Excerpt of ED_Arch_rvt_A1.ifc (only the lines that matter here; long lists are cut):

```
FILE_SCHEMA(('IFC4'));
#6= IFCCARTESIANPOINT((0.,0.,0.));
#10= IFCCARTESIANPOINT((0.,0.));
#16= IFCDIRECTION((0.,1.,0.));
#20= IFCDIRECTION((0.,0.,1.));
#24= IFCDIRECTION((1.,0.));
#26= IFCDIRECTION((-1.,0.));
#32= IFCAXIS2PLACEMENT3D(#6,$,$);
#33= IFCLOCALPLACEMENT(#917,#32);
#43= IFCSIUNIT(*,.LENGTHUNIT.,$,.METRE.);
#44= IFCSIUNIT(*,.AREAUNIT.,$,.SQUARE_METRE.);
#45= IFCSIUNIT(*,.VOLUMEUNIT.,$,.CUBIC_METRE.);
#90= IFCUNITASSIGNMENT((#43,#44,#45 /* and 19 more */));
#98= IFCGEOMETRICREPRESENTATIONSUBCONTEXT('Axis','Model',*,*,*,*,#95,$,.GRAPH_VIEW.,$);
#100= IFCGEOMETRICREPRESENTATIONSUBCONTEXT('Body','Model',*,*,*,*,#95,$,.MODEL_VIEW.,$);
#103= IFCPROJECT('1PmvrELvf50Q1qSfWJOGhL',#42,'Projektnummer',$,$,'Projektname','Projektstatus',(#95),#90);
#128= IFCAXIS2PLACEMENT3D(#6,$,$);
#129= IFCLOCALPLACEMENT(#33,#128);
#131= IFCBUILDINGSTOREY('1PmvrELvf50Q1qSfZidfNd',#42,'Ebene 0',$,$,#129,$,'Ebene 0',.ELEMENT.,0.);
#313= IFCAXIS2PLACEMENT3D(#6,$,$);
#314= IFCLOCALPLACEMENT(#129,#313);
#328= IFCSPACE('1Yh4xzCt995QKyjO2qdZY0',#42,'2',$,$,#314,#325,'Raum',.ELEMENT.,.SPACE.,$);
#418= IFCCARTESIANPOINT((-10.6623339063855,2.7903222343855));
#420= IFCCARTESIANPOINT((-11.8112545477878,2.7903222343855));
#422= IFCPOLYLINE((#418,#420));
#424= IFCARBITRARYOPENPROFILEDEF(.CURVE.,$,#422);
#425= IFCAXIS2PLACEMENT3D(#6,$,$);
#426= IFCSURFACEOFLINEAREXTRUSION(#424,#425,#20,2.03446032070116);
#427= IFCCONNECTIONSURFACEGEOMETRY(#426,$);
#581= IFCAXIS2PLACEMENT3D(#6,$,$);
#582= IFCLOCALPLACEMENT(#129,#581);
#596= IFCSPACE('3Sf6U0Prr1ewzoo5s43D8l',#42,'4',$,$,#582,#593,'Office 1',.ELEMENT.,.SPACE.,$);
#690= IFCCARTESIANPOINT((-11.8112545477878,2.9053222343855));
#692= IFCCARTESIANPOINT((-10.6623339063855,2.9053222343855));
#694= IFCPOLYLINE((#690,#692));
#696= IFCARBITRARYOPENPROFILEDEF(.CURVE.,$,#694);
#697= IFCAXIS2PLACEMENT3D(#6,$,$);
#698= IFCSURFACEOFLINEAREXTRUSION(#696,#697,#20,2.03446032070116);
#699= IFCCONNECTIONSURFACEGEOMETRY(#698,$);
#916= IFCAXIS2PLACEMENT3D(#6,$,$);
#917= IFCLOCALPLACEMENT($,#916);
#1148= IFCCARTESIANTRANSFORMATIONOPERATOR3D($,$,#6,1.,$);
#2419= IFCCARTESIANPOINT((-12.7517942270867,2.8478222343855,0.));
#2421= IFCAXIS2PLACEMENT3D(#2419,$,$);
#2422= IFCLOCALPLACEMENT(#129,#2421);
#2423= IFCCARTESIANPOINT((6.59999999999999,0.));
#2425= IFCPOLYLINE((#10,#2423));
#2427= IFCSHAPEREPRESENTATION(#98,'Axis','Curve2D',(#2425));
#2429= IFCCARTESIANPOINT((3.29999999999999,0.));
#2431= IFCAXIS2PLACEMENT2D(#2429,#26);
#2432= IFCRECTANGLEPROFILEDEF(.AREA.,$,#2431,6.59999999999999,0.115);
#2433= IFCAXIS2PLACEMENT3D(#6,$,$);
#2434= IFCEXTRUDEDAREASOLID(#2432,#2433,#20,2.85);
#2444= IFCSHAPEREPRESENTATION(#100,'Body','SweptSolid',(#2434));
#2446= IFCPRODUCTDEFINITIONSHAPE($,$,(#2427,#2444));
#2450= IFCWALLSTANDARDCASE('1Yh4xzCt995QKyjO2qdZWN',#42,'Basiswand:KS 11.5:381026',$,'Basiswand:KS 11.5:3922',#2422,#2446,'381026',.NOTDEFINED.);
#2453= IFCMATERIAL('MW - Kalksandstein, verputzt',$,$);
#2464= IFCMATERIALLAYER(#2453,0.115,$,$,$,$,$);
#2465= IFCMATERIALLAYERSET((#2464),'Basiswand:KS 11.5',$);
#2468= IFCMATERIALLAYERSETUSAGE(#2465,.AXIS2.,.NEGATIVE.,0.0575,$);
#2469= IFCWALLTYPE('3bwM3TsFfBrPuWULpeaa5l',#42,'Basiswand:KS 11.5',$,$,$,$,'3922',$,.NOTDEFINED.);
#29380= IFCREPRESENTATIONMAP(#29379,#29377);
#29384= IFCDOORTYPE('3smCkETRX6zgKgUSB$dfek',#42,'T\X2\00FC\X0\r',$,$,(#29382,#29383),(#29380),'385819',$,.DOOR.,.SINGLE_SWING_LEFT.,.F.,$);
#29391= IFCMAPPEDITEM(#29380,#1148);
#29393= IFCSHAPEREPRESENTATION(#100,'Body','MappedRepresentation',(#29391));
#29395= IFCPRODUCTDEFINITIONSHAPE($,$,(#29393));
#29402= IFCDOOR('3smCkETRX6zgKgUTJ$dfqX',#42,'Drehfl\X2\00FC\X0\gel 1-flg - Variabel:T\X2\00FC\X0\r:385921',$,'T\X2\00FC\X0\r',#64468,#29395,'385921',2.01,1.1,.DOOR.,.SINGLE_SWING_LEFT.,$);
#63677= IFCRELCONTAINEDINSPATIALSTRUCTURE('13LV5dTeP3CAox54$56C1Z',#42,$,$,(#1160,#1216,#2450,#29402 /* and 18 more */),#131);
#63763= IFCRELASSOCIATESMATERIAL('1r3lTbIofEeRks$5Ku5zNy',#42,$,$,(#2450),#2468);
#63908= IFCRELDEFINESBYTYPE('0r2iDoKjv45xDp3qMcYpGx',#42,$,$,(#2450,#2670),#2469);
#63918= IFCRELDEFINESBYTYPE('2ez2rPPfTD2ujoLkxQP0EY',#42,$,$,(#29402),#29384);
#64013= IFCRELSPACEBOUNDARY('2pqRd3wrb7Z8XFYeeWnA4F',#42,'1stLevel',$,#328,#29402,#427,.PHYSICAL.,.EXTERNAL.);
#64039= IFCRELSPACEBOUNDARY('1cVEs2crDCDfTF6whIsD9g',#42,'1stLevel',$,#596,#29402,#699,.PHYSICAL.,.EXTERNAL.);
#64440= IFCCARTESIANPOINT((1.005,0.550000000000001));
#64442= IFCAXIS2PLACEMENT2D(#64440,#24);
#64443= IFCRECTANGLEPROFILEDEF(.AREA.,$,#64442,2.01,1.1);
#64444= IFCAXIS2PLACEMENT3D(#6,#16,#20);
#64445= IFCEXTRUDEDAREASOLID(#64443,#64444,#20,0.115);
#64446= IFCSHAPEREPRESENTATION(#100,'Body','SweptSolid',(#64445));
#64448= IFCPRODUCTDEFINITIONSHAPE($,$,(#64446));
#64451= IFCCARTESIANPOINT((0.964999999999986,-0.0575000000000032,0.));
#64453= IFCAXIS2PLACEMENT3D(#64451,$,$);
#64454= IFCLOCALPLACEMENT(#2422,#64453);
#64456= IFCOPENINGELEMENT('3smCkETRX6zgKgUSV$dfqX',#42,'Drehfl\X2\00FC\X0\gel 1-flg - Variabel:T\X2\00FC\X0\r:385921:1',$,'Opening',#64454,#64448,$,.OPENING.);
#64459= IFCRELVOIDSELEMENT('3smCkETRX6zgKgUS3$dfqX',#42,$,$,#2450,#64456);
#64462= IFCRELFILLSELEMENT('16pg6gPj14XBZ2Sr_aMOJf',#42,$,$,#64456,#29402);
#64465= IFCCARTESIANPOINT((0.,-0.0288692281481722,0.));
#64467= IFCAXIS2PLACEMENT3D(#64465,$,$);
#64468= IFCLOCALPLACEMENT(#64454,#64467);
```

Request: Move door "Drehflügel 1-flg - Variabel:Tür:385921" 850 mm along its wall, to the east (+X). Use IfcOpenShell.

```python
import numpy as np
import ifcopenshell
import ifcopenshell.api.geometry
import ifcopenshell.util.placement

model = ifcopenshell.open("ED_Arch_rvt_A1.ifc")

door = model.by_id(29402)
opening = door.FillsVoids[0].RelatingOpeningElement
wall = opening.VoidsElements[0].RelatingBuildingElement

wall_matrix = ifcopenshell.util.placement.get_local_placement(wall.ObjectPlacement)
shift = wall_matrix[:3, 0] * 0.85
before = ifcopenshell.util.placement.get_local_placement(door.ObjectPlacement)[:3, 3].copy()

# The door is placed relative to its opening, so it follows when the opening moves.
matrix = ifcopenshell.util.placement.get_local_placement(opening.ObjectPlacement)
matrix[:3, 3] += shift
ifcopenshell.api.geometry.edit_object_placement(
    model, product=opening, matrix=matrix, is_si=False, should_transform_children=True
)

# Space boundary surfaces are stored in each space's coordinates; move them too.
for rel in door.ProvidesBoundaries:
    if not rel.ConnectionGeometry:
        continue
    surface = rel.ConnectionGeometry.SurfaceOnRelatingElement
    space_matrix = ifcopenshell.util.placement.get_local_placement(rel.RelatingSpace.ObjectPlacement)
    point = np.array(surface.Position.Location.Coordinates) + space_matrix[:3, :3].T @ shift
    surface.Position = model.createIfcAxis2Placement3D(
        model.createIfcCartesianPoint(point.tolist()), surface.Position.Axis, surface.Position.RefDirection
    )

after = ifcopenshell.util.placement.get_local_placement(door.ObjectPlacement)[:3, 3]
print("door moved by", (after - before).round(3) + 0.0)

model.write("ED_Arch_rvt_A1_edited.ifc")
```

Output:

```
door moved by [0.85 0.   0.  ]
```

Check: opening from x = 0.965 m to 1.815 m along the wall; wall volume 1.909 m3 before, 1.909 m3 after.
